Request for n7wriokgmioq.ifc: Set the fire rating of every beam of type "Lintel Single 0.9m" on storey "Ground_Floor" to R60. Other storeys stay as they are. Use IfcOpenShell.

First a look at what the model holds.

```python
import ifcopenshell
import ifcopenshell.util.element

model = ifcopenshell.open("n7wriokgmioq.ifc")
print(model.schema)
storey = next(s for s in model.by_type("IfcBuildingStorey") if s.Name == "Ground_Floor")
beams = [e for e in ifcopenshell.util.element.get_decomposition(storey) if e.is_a("IfcBeam")]
seen = {}
for e in beams:
    element_type = ifcopenshell.util.element.get_type(e)
    key = (element_type.Name if element_type != e and element_type else None, ifcopenshell.util.element.get_pset(e, "Pset_BeamCommon", "FireRating"))
    seen[key] = seen.get(key, 0) + 1
for (name, value), count in sorted(seen.items(), key=str):
    print(count, "x", name, "|", value)
```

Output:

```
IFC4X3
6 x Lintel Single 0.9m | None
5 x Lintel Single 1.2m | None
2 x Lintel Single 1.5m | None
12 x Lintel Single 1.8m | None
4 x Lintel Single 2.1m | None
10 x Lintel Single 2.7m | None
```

```python
import ifcopenshell
import ifcopenshell.api.pset
import ifcopenshell.util.element

model = ifcopenshell.open("n7wriokgmioq.ifc")

storey = next(s for s in model.by_type("IfcBuildingStorey") if s.Name == "Ground_Floor")
beams = [e for e in ifcopenshell.util.element.get_decomposition(storey) if e.is_a("IfcBeam")]

count = 0
for e in beams:
    element_type = ifcopenshell.util.element.get_type(e)
    if element_type in (None, e) or element_type.Name != "Lintel Single 0.9m":
        continue
    # add_pset returns the element's existing set when there is one.
    pset = ifcopenshell.api.pset.add_pset(model, product=e, name="Pset_BeamCommon")
    ifcopenshell.api.pset.edit_pset(model, pset=pset, properties={"FireRating": "R60"})
    count += 1

print(count, "beams updated")

model.write("n7wriokgmioq-out.ifc")
```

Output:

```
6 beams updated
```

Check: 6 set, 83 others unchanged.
